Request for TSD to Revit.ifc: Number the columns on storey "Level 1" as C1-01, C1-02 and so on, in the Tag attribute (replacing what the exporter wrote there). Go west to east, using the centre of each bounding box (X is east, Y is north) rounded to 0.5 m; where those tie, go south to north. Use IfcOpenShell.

First a look at what the model holds.

```python
import ifcopenshell
import ifcopenshell.util.element
import ifcopenshell.util.placement

model = ifcopenshell.open("TSD to Revit.ifc")
print(model.schema)
storey = next(s for s in model.by_type("IfcBuildingStorey") if s.Name == "Level 1")
columns = [e for e in ifcopenshell.util.element.get_decomposition(storey) if e.is_a("IfcColumn")]
for e in sorted(columns, key=lambda e: e.id()):
    origin = ifcopenshell.util.placement.get_local_placement(e.ObjectPlacement)[:3, 3]
    print(e.id(), e.Tag, e.Name, origin.round(2) + 0.0, sep=" | ")
```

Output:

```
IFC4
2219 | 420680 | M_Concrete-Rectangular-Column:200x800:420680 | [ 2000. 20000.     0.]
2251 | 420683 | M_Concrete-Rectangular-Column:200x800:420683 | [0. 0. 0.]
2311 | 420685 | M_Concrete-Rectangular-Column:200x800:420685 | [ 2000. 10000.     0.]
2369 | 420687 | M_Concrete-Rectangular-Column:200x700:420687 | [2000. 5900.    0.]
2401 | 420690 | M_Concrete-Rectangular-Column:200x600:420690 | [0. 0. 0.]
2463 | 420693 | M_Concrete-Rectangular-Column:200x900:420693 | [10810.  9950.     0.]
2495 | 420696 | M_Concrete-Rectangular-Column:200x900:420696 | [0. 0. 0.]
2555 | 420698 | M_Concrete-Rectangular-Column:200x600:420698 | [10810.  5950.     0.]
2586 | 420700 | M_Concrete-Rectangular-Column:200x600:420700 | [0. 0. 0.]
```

```python
import ifcopenshell
import ifcopenshell.geom
import ifcopenshell.util.element
import ifcopenshell.util.shape

model = ifcopenshell.open("TSD to Revit.ifc")
settings = ifcopenshell.geom.settings()
settings.set("use-world-coords", True)


def centre(element):
    shape = ifcopenshell.geom.create_shape(settings, element)
    return ifcopenshell.util.shape.get_bbox_centroid(shape.geometry)


storey = next(s for s in model.by_type("IfcBuildingStorey") if s.Name == "Level 1")
columns = [e for e in ifcopenshell.util.element.get_decomposition(storey) if e.is_a("IfcColumn")]

# Insertion points can sit at a corner or the storey origin, so sort by the geometry (in metres).
centres = {e: centre(e) for e in columns}
columns.sort(key=lambda e: (round(centres[e][0] / 0.5), centres[e][1]))

for i, e in enumerate(columns, start=1):
    number = f"C1-{i:02d}"
    e.Tag = number
    print(e.id(), number)

model.write("TSD to Revit_updated.ifc")
```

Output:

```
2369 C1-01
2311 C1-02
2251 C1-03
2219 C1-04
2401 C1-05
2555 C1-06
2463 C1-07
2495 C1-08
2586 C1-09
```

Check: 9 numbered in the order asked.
